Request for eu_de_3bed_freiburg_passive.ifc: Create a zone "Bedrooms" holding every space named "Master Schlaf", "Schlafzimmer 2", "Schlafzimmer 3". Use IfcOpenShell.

First a look at what the model holds.

```python
import ifcopenshell

model = ifcopenshell.open("eu_de_3bed_freiburg_passive.ifc")
print(model.schema)
seen = {}
for space in model.by_type("IfcSpace"):
    seen[space.LongName] = seen.get(space.LongName, 0) + 1
for name, count in sorted(seen.items(), key=str):
    print(count, "x", name)
print("zones:", [z.Name for z in model.by_type("IfcZone")][:20])
```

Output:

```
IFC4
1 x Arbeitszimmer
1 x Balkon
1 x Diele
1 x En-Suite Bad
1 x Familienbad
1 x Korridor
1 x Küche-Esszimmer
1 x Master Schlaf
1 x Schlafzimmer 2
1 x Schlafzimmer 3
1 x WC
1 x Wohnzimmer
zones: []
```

```python
import ifcopenshell
import ifcopenshell.api.group
import ifcopenshell.api.root

model = ifcopenshell.open("eu_de_3bed_freiburg_passive.ifc")

names = {"Master Schlaf", "Schlafzimmer 2", "Schlafzimmer 3"}
spaces = [s for s in model.by_type("IfcSpace") if s.LongName in names]

zone = ifcopenshell.api.root.create_entity(model, ifc_class="IfcZone", name="Bedrooms")
ifcopenshell.api.group.assign_group(model, products=spaces, group=zone)
print(len(spaces), "spaces in", zone.Name)

model.write("eu_de_3bed_freiburg_passive_v2.ifc")
```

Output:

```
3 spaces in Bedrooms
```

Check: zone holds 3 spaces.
